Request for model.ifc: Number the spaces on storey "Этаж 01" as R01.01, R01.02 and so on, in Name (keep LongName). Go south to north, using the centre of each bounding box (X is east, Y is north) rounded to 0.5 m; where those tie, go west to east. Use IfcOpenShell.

First a look at what the model holds.

```python
import ifcopenshell
import ifcopenshell.util.element
import ifcopenshell.util.placement

model = ifcopenshell.open("model.ifc")
print(model.schema)
storey = next(s for s in model.by_type("IfcBuildingStorey") if s.Name == "Этаж 01")
spaces = [e for e in ifcopenshell.util.element.get_decomposition(storey) if e.is_a("IfcSpace")]
for e in sorted(spaces, key=lambda e: e.id()):
    origin = ifcopenshell.util.placement.get_local_placement(e.ObjectPlacement)[:3, 3]
    print(e.id(), e.Name, e.LongName, origin.round(2) + 0.0, sep=" | ")
```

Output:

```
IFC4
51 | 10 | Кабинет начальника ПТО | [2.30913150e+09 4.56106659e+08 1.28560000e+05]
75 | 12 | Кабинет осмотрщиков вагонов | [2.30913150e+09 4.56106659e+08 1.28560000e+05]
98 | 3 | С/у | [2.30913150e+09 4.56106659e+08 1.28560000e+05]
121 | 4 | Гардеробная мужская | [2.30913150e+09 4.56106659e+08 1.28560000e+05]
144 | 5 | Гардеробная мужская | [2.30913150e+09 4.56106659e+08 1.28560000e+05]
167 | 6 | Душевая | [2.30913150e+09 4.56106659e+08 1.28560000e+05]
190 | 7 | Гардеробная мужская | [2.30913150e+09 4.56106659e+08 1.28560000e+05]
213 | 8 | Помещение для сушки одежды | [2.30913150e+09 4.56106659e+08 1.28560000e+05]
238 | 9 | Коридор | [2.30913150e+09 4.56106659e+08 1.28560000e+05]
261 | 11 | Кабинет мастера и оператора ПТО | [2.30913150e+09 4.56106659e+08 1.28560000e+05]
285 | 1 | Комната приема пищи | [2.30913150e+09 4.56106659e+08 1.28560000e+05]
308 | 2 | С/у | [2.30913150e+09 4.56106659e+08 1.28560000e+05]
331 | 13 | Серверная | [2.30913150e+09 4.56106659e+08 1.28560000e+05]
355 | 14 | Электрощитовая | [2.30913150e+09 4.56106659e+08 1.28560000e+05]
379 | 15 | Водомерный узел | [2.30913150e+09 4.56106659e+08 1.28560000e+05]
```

```python
import ifcopenshell
import ifcopenshell.geom
import ifcopenshell.util.element
import ifcopenshell.util.shape

model = ifcopenshell.open("model.ifc")
settings = ifcopenshell.geom.settings()
settings.set("use-world-coords", True)


def centre(element):
    shape = ifcopenshell.geom.create_shape(settings, element)
    return ifcopenshell.util.shape.get_bbox_centroid(shape.geometry)


storey = next(s for s in model.by_type("IfcBuildingStorey") if s.Name == "Этаж 01")
spaces = [e for e in ifcopenshell.util.element.get_decomposition(storey) if e.is_a("IfcSpace")]

# Insertion points can sit at a corner or the storey origin, so sort by the geometry (in metres).
centres = {e: centre(e) for e in spaces}
spaces.sort(key=lambda e: (round(centres[e][1] / 0.5), centres[e][0]))

for i, e in enumerate(spaces, start=1):
    number = f"R01.{i:02d}"
    e.Name = number
    print(e.id(), number)

model.write("model_rev.ifc")
```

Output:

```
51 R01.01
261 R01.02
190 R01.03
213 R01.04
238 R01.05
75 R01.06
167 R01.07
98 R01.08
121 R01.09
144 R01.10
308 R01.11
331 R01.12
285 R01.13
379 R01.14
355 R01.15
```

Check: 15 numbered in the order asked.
